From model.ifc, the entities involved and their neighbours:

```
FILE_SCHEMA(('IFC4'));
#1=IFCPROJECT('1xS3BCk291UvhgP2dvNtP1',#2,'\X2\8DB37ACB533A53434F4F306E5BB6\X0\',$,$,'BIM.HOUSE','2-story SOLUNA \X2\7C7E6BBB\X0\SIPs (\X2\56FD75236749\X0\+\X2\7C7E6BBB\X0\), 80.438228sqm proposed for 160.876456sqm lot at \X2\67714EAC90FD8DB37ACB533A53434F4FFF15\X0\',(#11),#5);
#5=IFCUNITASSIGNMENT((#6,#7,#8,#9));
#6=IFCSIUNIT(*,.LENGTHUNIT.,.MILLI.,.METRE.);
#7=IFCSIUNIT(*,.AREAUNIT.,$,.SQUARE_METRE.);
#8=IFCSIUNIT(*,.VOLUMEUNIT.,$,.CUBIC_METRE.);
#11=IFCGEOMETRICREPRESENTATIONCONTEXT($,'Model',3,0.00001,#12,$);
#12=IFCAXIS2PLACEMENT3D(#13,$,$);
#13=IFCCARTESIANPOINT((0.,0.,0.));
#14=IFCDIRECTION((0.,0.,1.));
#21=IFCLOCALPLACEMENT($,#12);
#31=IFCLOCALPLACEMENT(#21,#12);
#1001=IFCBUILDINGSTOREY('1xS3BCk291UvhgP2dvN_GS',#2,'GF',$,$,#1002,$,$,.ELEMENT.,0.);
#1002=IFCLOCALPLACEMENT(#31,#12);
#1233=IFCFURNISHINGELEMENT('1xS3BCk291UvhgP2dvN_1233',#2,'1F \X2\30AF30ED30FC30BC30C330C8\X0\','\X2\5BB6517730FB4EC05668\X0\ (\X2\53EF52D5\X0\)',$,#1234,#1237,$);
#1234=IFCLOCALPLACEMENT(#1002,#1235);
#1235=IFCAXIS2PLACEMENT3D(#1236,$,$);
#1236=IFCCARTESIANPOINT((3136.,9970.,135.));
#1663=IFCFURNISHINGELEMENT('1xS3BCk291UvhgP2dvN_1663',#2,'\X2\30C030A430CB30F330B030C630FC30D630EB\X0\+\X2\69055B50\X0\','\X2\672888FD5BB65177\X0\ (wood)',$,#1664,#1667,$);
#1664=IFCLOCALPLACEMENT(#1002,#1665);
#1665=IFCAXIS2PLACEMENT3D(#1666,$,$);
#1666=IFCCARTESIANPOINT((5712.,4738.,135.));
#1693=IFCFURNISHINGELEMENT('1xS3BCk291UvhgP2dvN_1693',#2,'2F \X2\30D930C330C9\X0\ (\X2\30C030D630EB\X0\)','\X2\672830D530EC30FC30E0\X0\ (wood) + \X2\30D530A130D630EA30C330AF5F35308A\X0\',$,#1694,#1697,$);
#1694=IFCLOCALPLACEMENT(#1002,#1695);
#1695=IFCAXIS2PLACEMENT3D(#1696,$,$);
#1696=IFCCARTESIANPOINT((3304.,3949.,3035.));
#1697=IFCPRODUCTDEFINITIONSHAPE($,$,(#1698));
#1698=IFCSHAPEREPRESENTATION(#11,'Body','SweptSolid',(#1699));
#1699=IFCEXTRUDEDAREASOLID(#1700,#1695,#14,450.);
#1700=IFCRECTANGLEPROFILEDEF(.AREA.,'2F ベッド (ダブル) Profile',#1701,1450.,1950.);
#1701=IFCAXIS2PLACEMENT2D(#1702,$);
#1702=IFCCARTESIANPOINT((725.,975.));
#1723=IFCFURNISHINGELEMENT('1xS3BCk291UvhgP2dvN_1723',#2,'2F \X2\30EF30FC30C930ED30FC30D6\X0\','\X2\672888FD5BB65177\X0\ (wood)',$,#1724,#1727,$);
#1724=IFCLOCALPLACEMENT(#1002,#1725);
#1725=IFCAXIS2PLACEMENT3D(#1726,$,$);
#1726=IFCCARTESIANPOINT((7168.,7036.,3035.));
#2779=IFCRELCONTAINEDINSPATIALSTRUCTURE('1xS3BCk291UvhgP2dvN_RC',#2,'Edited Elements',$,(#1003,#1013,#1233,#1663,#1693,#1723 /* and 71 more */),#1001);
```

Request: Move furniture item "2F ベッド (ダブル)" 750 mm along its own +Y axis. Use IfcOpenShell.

```python
import ifcopenshell
import ifcopenshell.api.geometry
import ifcopenshell.util.placement
import ifcopenshell.util.unit

model = ifcopenshell.open("model.ifc")
unit_scale = ifcopenshell.util.unit.calculate_unit_scale(model)

item = model.by_id(1693)
matrix = ifcopenshell.util.placement.get_local_placement(item.ObjectPlacement)
matrix[:3, 3] += matrix[:3, 1] * 0.75 / unit_scale
ifcopenshell.api.geometry.edit_object_placement(model, product=item, matrix=matrix, is_si=False)

print(ifcopenshell.util.placement.get_local_placement(item.ObjectPlacement).round(3) + 0.0)

model.write("model_v2.ifc")
```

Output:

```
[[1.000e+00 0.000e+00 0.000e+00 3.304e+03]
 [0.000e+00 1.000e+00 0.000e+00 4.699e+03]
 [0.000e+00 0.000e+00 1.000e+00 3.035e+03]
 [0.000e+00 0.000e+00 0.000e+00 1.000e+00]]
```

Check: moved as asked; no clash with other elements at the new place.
